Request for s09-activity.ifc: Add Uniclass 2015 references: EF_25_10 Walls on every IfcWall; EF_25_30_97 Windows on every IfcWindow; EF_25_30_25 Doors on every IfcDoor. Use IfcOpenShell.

First a look at what the model holds.

```python
import ifcopenshell

model = ifcopenshell.open("s09-activity.ifc")
print(model.schema)
print("classifications:", [c.Name for c in model.by_type("IfcClassification")])
for ifc_class in ("IfcDoor", "IfcRoof", "IfcStair", "IfcWall", "IfcWindow"):
    print(ifc_class, len(model.by_type(ifc_class)))
```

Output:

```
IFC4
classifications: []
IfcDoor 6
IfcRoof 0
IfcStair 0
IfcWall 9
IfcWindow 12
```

```python
import ifcopenshell
import ifcopenshell.api.classification

model = ifcopenshell.open("s09-activity.ifc")

system = ifcopenshell.api.classification.add_classification(model, classification="Uniclass 2015")

codes = {
    "IfcWall": ("EF_25_10", "Walls"),
    "IfcWindow": ("EF_25_30_97", "Windows"),
    "IfcDoor": ("EF_25_30_25", "Doors"),
}
for ifc_class, (code, name) in codes.items():
    products = model.by_type(ifc_class)
    ifcopenshell.api.classification.add_reference(
        model, products=products, classification=system, identification=code, name=name
    )
    print(code, len(products))

model.write("s09-activity_rev.ifc")
```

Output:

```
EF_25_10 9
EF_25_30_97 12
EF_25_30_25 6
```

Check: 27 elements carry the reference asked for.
